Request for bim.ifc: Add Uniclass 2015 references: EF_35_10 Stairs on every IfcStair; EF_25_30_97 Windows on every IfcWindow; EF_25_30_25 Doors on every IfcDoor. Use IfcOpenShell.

First a look at what the model holds.

```python
import ifcopenshell

model = ifcopenshell.open("bim.ifc")
print(model.schema)
print("classifications:", [c.Name for c in model.by_type("IfcClassification")])
for ifc_class in ("IfcDoor", "IfcRoof", "IfcStair", "IfcWall", "IfcWindow"):
    print(ifc_class, len(model.by_type(ifc_class)))
```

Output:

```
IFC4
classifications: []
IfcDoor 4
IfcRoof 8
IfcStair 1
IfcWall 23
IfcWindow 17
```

```python
import ifcopenshell
import ifcopenshell.api.classification

model = ifcopenshell.open("bim.ifc")

system = ifcopenshell.api.classification.add_classification(model, classification="Uniclass 2015")

codes = {
    "IfcStair": ("EF_35_10", "Stairs"),
    "IfcWindow": ("EF_25_30_97", "Windows"),
    "IfcDoor": ("EF_25_30_25", "Doors"),
}
for ifc_class, (code, name) in codes.items():
    products = model.by_type(ifc_class)
    ifcopenshell.api.classification.add_reference(
        model, products=products, classification=system, identification=code, name=name
    )
    print(code, len(products))

model.write("bim_edited.ifc")
```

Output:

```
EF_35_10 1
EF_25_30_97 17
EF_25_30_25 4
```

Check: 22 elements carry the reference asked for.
